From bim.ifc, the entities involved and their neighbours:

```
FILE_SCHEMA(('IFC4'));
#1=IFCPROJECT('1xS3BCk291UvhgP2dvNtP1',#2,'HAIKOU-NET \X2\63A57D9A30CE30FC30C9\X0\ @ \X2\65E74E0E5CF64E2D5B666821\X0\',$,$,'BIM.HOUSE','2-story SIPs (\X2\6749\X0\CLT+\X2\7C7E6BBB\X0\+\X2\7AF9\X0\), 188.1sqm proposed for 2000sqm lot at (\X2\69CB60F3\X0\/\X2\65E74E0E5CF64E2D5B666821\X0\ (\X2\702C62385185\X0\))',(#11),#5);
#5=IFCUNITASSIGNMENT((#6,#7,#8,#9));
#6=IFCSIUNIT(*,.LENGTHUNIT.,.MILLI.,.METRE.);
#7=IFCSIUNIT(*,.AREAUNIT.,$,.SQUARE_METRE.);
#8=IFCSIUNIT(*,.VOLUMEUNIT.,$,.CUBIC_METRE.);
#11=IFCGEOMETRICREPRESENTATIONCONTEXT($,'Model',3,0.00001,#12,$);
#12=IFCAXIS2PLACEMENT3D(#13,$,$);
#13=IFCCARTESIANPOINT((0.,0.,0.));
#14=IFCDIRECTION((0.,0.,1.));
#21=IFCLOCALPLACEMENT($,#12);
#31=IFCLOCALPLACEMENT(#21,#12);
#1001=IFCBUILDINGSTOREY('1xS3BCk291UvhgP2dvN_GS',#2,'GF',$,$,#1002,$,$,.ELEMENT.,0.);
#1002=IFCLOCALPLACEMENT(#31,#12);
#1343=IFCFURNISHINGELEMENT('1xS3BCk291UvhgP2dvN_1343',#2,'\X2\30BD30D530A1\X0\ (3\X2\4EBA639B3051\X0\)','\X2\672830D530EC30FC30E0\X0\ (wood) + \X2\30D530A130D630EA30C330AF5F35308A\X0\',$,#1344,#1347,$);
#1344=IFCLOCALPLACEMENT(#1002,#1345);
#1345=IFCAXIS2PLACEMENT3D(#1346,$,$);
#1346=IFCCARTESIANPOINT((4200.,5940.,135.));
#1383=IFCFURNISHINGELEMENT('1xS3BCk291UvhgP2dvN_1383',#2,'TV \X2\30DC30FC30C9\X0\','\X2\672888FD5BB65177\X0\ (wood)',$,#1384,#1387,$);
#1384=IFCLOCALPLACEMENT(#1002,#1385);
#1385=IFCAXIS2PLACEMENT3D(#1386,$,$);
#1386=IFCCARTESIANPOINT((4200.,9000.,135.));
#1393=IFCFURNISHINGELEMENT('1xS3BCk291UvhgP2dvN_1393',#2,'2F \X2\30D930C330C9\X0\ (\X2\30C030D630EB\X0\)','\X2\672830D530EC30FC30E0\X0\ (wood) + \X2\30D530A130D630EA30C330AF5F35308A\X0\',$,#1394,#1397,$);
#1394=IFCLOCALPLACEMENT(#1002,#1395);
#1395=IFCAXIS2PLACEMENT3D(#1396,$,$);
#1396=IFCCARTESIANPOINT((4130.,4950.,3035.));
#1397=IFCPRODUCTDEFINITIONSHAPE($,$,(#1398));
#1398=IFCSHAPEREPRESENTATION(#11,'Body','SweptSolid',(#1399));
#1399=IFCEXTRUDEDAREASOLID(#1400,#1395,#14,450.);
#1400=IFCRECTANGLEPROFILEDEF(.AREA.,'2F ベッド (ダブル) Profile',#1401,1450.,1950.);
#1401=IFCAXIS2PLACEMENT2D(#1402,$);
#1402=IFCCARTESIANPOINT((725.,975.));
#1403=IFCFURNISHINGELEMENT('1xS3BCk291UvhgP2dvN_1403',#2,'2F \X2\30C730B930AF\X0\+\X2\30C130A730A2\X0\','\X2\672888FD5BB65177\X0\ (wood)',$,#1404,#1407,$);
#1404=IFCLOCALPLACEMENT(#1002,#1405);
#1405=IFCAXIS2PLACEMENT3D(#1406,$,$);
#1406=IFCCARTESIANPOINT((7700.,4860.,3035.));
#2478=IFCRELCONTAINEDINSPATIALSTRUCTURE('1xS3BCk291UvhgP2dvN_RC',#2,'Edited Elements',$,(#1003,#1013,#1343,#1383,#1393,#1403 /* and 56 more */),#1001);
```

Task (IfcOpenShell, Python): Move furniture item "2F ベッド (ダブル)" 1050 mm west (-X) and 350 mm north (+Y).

```python
import ifcopenshell
import ifcopenshell.api.geometry
import ifcopenshell.util.placement
import ifcopenshell.util.unit

model = ifcopenshell.open("bim.ifc")
unit_scale = ifcopenshell.util.unit.calculate_unit_scale(model)

item = model.by_id(1393)
matrix = ifcopenshell.util.placement.get_local_placement(item.ObjectPlacement)
matrix[0, 3] -= 1.05 / unit_scale
matrix[1, 3] += 0.35 / unit_scale
ifcopenshell.api.geometry.edit_object_placement(model, product=item, matrix=matrix, is_si=False)

print(ifcopenshell.util.placement.get_local_placement(item.ObjectPlacement).round(3) + 0.0)

model.write("bim-out.ifc")
```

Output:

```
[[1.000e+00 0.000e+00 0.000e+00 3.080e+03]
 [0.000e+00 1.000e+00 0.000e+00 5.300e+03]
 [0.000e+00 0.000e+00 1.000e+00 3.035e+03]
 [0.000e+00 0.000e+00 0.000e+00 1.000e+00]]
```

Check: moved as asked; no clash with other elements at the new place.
